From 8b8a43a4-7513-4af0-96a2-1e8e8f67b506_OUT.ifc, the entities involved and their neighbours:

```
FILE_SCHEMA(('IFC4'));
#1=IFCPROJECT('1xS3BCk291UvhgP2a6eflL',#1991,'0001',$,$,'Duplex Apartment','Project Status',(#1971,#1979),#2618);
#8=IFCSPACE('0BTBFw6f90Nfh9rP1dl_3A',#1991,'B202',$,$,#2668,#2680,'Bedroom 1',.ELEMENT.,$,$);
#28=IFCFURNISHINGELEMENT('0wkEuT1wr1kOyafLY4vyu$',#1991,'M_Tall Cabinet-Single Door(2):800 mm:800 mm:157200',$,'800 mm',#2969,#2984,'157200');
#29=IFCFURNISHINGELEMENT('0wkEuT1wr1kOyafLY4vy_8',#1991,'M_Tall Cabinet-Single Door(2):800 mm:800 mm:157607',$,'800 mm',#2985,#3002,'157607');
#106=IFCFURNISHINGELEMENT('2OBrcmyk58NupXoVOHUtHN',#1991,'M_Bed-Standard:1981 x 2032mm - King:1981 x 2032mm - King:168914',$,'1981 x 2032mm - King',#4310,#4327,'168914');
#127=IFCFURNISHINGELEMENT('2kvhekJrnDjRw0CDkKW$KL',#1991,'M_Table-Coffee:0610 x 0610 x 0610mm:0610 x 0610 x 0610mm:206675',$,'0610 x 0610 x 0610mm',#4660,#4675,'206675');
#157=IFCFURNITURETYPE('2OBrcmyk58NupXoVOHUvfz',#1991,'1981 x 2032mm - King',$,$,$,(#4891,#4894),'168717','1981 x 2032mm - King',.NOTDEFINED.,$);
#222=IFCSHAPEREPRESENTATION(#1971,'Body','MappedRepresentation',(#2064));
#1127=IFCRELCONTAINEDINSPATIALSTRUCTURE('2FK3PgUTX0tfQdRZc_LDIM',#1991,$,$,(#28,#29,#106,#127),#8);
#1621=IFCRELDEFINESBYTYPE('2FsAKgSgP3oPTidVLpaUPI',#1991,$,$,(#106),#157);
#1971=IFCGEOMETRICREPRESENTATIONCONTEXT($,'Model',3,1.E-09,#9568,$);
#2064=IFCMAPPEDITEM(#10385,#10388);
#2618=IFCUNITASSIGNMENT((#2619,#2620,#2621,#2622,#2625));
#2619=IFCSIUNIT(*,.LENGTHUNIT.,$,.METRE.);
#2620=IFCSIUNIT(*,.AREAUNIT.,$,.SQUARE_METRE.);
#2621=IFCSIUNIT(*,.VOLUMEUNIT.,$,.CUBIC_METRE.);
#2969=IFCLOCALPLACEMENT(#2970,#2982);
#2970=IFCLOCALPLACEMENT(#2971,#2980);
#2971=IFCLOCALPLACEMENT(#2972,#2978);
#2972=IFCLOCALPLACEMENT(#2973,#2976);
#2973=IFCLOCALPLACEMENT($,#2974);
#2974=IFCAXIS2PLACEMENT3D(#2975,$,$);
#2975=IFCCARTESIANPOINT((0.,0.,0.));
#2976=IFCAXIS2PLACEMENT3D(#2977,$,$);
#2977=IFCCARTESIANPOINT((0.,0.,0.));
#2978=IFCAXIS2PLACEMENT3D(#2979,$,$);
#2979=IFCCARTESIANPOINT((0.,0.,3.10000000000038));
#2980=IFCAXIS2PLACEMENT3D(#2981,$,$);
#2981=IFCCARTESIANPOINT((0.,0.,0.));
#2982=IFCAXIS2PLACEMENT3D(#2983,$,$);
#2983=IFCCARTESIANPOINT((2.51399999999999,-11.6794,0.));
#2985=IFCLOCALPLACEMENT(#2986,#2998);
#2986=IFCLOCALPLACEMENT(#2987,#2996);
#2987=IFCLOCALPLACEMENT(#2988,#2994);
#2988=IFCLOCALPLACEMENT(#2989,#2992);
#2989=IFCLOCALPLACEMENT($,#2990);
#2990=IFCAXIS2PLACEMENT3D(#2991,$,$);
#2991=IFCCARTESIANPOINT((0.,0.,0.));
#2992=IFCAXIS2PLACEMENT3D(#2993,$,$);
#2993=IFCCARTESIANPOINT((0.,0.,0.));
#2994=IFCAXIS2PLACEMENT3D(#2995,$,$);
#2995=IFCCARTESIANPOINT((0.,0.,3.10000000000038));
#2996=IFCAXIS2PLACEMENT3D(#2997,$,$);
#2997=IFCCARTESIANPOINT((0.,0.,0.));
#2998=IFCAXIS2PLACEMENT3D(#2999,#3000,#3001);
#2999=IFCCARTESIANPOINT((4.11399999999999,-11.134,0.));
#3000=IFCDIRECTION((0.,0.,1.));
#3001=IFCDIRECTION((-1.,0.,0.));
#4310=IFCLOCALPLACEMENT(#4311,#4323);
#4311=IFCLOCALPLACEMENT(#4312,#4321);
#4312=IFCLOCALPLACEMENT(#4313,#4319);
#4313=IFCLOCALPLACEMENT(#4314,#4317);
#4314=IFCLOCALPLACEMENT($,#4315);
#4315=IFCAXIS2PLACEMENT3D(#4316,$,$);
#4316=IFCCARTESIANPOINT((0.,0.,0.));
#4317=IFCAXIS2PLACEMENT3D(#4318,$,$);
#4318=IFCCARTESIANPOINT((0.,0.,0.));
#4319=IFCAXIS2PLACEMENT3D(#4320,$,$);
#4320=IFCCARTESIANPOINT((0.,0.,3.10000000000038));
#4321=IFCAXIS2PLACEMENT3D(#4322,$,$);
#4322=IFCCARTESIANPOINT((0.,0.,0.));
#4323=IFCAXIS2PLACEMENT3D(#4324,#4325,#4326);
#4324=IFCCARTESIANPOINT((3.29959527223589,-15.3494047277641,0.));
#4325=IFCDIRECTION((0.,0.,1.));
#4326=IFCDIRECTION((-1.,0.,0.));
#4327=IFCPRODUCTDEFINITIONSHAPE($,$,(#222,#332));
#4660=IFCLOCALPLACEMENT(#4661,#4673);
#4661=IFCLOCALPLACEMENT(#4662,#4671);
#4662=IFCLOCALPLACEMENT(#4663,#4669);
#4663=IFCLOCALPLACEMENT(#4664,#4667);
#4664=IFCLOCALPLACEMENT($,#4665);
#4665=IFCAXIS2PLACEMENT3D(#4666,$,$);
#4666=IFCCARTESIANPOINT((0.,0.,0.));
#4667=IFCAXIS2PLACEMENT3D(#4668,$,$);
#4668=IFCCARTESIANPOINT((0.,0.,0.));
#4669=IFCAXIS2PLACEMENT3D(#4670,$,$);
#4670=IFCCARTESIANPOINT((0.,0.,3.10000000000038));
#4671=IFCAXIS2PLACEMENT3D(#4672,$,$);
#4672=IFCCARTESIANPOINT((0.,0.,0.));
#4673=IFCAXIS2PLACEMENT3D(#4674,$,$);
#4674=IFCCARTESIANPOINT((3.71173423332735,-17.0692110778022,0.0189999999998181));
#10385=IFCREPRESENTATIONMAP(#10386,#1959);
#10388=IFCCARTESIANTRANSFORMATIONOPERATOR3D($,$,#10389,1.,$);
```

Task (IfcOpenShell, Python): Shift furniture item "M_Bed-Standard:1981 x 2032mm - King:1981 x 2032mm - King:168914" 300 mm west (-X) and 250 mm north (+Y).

```python
import ifcopenshell
import ifcopenshell.api.geometry
import ifcopenshell.util.placement

model = ifcopenshell.open("8b8a43a4-7513-4af0-96a2-1e8e8f67b506_OUT.ifc")

item = model.by_guid("2OBrcmyk58NupXoVOHUtHN")
matrix = ifcopenshell.util.placement.get_local_placement(item.ObjectPlacement)
matrix[0, 3] -= 0.3
matrix[1, 3] += 0.25
ifcopenshell.api.geometry.edit_object_placement(model, product=item, matrix=matrix, is_si=False)

print(ifcopenshell.util.placement.get_local_placement(item.ObjectPlacement).round(3) + 0.0)

model.write("8b8a43a4-7513-4af0-96a2-1e8e8f67b506_OUT_v2.ifc")
```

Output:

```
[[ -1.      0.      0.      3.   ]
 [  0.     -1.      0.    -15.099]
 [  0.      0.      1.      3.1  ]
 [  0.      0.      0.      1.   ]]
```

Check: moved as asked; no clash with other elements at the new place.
